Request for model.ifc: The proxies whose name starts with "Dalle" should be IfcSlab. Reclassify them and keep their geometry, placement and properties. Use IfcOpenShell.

First a look at what the model holds.

```python
import re

import ifcopenshell

model = ifcopenshell.open("model.ifc")
print(model.schema)
seen = {}
for e in model.by_type("IfcBuildingElementProxy"):
    name = re.sub(r":\d+(:\d+)?$", "", e.Name or "")  # drop the element id that some exporters append
    seen[name] = seen.get(name, 0) + 1
for name, count in sorted(seen.items()):
    print(count, "x", name)
```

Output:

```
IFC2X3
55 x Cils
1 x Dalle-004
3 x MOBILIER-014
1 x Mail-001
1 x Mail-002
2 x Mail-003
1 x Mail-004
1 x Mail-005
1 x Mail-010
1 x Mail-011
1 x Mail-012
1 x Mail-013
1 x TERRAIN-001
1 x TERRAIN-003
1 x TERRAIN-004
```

```python
import ifcopenshell
import ifcopenshell.api.root

model = ifcopenshell.open("model.ifc")

proxies = [e.id() for e in model.by_type("IfcBuildingElementProxy") if (e.Name or "").startswith("Dalle")]
for step_id in proxies:
    proxy = model.by_id(step_id)
    # Reclassifying a typed element also reclassifies its type and the type's other occurrences.
    if proxy.is_a("IfcBuildingElementProxy"):
        ifcopenshell.api.root.reassign_class(model, product=proxy, ifc_class="IfcSlab", predefined_type="FLOOR")

print(sum(model.by_id(i).is_a("IfcSlab") for i in proxies), "reclassified")

model.write("model_rev.ifc")
```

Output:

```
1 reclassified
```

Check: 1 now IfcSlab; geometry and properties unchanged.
